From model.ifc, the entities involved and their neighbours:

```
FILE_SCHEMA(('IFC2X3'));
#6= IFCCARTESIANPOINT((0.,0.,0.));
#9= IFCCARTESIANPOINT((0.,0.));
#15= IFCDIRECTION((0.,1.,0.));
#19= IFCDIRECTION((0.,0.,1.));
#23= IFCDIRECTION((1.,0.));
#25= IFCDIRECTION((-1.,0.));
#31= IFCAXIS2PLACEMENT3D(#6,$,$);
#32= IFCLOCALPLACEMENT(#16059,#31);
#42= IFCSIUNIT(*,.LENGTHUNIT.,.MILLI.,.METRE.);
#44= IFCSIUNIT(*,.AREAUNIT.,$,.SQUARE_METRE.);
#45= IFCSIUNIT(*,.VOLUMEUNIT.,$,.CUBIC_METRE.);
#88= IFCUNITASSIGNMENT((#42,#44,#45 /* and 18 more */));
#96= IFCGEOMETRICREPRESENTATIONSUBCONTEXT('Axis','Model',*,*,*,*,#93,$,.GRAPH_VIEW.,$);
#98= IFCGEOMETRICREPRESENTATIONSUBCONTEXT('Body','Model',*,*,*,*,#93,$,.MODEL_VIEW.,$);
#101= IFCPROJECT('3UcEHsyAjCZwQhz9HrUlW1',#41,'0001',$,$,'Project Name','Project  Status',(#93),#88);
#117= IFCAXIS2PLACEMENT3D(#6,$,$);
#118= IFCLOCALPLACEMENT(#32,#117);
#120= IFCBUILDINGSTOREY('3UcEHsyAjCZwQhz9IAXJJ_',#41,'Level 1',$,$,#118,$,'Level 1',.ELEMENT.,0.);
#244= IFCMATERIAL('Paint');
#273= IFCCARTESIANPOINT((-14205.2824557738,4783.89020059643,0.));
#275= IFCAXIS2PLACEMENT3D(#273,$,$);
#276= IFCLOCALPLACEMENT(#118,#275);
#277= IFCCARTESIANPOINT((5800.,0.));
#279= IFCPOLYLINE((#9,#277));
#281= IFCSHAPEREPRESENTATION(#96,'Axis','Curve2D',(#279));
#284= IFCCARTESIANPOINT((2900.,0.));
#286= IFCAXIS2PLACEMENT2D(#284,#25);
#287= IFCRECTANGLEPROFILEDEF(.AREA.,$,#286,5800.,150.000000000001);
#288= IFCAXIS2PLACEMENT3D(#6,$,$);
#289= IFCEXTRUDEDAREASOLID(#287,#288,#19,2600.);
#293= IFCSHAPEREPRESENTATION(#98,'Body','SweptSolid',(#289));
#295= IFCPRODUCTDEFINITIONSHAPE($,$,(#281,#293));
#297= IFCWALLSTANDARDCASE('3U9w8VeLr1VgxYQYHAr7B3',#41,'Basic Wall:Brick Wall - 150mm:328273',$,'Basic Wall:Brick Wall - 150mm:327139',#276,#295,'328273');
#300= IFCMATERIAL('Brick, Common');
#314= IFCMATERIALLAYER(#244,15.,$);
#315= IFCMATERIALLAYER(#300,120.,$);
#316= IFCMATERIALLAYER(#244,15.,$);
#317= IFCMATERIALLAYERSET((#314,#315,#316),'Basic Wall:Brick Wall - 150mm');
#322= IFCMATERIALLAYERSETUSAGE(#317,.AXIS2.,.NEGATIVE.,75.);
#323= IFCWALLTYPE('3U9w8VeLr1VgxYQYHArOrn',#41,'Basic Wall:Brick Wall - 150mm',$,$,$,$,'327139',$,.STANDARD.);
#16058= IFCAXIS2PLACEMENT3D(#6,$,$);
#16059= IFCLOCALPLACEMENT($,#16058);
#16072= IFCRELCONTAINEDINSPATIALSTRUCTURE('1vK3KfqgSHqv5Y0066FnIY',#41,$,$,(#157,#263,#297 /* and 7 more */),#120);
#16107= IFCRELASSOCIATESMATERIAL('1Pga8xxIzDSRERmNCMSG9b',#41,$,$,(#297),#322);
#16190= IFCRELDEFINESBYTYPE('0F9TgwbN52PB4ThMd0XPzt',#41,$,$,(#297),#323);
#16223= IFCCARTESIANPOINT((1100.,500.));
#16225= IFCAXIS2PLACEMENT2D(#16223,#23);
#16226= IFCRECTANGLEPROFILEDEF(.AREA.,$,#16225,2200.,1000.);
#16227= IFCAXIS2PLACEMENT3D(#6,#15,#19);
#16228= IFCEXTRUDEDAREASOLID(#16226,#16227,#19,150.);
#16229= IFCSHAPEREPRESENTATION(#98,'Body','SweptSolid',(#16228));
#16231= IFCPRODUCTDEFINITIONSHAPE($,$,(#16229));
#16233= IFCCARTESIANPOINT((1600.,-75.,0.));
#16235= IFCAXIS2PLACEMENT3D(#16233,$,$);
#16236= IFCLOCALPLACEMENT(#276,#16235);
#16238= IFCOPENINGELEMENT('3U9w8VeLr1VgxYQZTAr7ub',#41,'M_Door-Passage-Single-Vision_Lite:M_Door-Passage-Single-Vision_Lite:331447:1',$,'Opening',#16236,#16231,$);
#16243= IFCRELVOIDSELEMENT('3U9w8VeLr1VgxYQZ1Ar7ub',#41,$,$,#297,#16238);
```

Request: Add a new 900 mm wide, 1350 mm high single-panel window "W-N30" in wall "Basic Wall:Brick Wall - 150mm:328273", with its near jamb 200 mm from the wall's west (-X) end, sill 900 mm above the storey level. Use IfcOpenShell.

```python
import numpy as np
import ifcopenshell
import ifcopenshell.api.feature
import ifcopenshell.api.geometry
import ifcopenshell.api.root
import ifcopenshell.api.spatial
import ifcopenshell.api.type
import ifcopenshell.geom
import ifcopenshell.util.element
import ifcopenshell.util.placement
import ifcopenshell.util.representation
import ifcopenshell.util.shape
import ifcopenshell.util.unit

model = ifcopenshell.open("model.ifc")
unit_scale = ifcopenshell.util.unit.calculate_unit_scale(model)
settings = ifcopenshell.geom.settings()


def volume(element):
    """Net volume in cubic metres, openings subtracted."""
    shape = ifcopenshell.geom.create_shape(settings, element)
    return ifcopenshell.util.shape.get_volume(shape.geometry)


wall = model.by_id(297)
storey = ifcopenshell.util.element.get_container(wall, ifc_class="IfcBuildingStorey")
context = ifcopenshell.util.representation.get_context(model, "Model", "Body", "MODEL_VIEW")
before = volume(wall)

width, height, from_end, sill = 0.9, 1.35, 0.2, 0.9  # metres

# The wall runs along its own X axis, and the end named is its -X end.
wall_shape = ifcopenshell.geom.create_shape(settings, wall)
x, y, z = ifcopenshell.util.shape.get_vertices(wall_shape.geometry).T
start = x.min() + from_end
face, thickness = float(y.min()), float(y.max() - y.min())
wall_matrix = ifcopenshell.util.placement.get_local_placement(wall.ObjectPlacement)
level = ifcopenshell.util.placement.get_local_placement(storey.ObjectPlacement)[2, 3]


def in_wall(x, y):
    """Placement at x, y metres in the wall's axes, at sill height."""
    matrix = wall_matrix.copy()
    matrix[:, 3] = wall_matrix @ np.array([x / unit_scale, y / unit_scale, 0.0, 1.0])
    matrix[2, 3] = level + sill / unit_scale
    return matrix


# Opening: a box that overshoots both wall faces by 50 mm.
opening = ifcopenshell.api.root.create_entity(model, ifc_class="IfcOpeningElement")
box = ifcopenshell.api.geometry.add_wall_representation(
    model, context=context, length=width, height=height, thickness=thickness + 0.1
)
ifcopenshell.api.geometry.assign_representation(model, product=opening, representation=box)
ifcopenshell.api.geometry.edit_object_placement(model, product=opening, matrix=in_wall(start, face - 0.05), is_si=False)
ifcopenshell.api.feature.add_feature(model, feature=opening, element=wall)

window = ifcopenshell.api.root.create_entity(model, ifc_class="IfcWindow", name="W-N30")
window.OverallWidth, window.OverallHeight = width / unit_scale, height / unit_scale
body = ifcopenshell.api.geometry.add_window_representation(
    model,
    context=context,
    overall_width=window.OverallWidth,
    overall_height=window.OverallHeight,
    partition_type="SINGLE_PANEL",
)
ifcopenshell.api.geometry.assign_representation(model, product=window, representation=body)
ifcopenshell.api.spatial.assign_container(model, products=[window], relating_structure=storey)
fills = ifcopenshell.api.feature.add_filling(model, opening=opening, element=window)
fills.OwnerHistory = window.OwnerHistory  # required in IFC2X3

# IFC2X3 keeps the operation on the window style.
style = ifcopenshell.api.root.create_entity(model, ifc_class="IfcWindowStyle", name="W-N30")
style.OperationType, style.ConstructionType = "SINGLE_PANEL", "NOTDEFINED"
style.ParameterTakesPrecedence = style.Sizeable = False
ifcopenshell.api.type.assign_type(model, related_objects=[window], relating_type=style)

# Centre the window in the wall's thickness.
ifcopenshell.api.geometry.edit_object_placement(model, product=window, matrix=in_wall(start, face), is_si=False)
window_shape = ifcopenshell.geom.create_shape(settings, window)
depth = ifcopenshell.util.shape.get_vertices(window_shape.geometry)[:, 1]
offset = face + thickness / 2 - (depth.min() + depth.max()) / 2
ifcopenshell.api.geometry.edit_object_placement(model, product=window, matrix=in_wall(start, offset), is_si=False)

after = volume(wall)

print(f"wall volume {before:.3f} -> {after:.3f} m3")

model.write("model_v2.ifc")
```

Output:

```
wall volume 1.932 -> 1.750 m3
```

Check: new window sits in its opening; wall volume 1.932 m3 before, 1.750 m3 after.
